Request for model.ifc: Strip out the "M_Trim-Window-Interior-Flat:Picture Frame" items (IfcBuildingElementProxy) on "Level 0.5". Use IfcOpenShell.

First a look at what the model holds.

```python
import ifcopenshell
import ifcopenshell.util.element

model = ifcopenshell.open("model.ifc")
print(model.schema)
storey = next(s for s in model.by_type("IfcBuildingStorey") if s.Name == "Level 0.5")
proxies = [e for e in ifcopenshell.util.element.get_decomposition(storey) if e.is_a("IfcBuildingElementProxy")]
seen = {}
for e in proxies:
    element_type = ifcopenshell.util.element.get_type(e)
    name = element_type.Name if element_type not in (None, e) else None
    seen[name] = seen.get(name, 0) + 1
for name, count in sorted(seen.items(), key=str):
    print(count, "x", name)
```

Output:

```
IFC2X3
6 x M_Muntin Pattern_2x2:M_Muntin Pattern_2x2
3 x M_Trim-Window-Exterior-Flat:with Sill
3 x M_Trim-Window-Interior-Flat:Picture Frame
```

```python
import ifcopenshell
import ifcopenshell.api.root
import ifcopenshell.util.element

model = ifcopenshell.open("model.ifc")

storey = next(s for s in model.by_type("IfcBuildingStorey") if s.Name == "Level 0.5")
proxies = [e for e in ifcopenshell.util.element.get_decomposition(storey) if e.is_a("IfcBuildingElementProxy")]
targets = [e for e in proxies if (t := ifcopenshell.util.element.get_type(e)) not in (None, e) and t.Name == "M_Trim-Window-Interior-Flat:Picture Frame"]

for e in targets:
    ifcopenshell.api.root.remove_product(model, product=e)
print(len(targets), "removed")

model.write("model-out.ifc")
```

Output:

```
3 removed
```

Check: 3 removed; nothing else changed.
